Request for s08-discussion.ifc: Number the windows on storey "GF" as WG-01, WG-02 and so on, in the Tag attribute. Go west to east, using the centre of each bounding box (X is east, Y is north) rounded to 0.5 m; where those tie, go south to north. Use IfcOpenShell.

First a look at what the model holds.

```python
import ifcopenshell
import ifcopenshell.util.element
import ifcopenshell.util.placement

model = ifcopenshell.open("s08-discussion.ifc")
print(model.schema)
storey = next(s for s in model.by_type("IfcBuildingStorey") if s.Name == "GF")
windows = [e for e in ifcopenshell.util.element.get_decomposition(storey) if e.is_a("IfcWindow")]
for e in sorted(windows, key=lambda e: e.id()):
    origin = ifcopenshell.util.placement.get_local_placement(e.ObjectPlacement)[:3, 3]
    print(e.id(), e.Tag, e.Name, origin.round(2) + 0.0, sep=" | ")
```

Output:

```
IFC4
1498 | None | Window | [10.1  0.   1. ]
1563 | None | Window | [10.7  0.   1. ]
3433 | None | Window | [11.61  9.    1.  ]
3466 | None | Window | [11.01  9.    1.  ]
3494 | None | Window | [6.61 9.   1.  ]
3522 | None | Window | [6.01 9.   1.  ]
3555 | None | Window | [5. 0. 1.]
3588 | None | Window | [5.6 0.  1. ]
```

```python
import ifcopenshell
import ifcopenshell.geom
import ifcopenshell.util.element
import ifcopenshell.util.shape

model = ifcopenshell.open("s08-discussion.ifc")
settings = ifcopenshell.geom.settings()
settings.set("use-world-coords", True)


def centre(element):
    shape = ifcopenshell.geom.create_shape(settings, element)
    return ifcopenshell.util.shape.get_bbox_centroid(shape.geometry)


storey = next(s for s in model.by_type("IfcBuildingStorey") if s.Name == "GF")
windows = [e for e in ifcopenshell.util.element.get_decomposition(storey) if e.is_a("IfcWindow")]

# Insertion points can sit at a corner or the storey origin, so sort by the geometry (in metres).
centres = {e: centre(e) for e in windows}
windows.sort(key=lambda e: (round(centres[e][0] / 0.5), centres[e][1]))

for i, e in enumerate(windows, start=1):
    number = f"WG-{i:02d}"
    e.Tag = number
    print(e.id(), number)

model.write("s08-discussion-out.ifc")
```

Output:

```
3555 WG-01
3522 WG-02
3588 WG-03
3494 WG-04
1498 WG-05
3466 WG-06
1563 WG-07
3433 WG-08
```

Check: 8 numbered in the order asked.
